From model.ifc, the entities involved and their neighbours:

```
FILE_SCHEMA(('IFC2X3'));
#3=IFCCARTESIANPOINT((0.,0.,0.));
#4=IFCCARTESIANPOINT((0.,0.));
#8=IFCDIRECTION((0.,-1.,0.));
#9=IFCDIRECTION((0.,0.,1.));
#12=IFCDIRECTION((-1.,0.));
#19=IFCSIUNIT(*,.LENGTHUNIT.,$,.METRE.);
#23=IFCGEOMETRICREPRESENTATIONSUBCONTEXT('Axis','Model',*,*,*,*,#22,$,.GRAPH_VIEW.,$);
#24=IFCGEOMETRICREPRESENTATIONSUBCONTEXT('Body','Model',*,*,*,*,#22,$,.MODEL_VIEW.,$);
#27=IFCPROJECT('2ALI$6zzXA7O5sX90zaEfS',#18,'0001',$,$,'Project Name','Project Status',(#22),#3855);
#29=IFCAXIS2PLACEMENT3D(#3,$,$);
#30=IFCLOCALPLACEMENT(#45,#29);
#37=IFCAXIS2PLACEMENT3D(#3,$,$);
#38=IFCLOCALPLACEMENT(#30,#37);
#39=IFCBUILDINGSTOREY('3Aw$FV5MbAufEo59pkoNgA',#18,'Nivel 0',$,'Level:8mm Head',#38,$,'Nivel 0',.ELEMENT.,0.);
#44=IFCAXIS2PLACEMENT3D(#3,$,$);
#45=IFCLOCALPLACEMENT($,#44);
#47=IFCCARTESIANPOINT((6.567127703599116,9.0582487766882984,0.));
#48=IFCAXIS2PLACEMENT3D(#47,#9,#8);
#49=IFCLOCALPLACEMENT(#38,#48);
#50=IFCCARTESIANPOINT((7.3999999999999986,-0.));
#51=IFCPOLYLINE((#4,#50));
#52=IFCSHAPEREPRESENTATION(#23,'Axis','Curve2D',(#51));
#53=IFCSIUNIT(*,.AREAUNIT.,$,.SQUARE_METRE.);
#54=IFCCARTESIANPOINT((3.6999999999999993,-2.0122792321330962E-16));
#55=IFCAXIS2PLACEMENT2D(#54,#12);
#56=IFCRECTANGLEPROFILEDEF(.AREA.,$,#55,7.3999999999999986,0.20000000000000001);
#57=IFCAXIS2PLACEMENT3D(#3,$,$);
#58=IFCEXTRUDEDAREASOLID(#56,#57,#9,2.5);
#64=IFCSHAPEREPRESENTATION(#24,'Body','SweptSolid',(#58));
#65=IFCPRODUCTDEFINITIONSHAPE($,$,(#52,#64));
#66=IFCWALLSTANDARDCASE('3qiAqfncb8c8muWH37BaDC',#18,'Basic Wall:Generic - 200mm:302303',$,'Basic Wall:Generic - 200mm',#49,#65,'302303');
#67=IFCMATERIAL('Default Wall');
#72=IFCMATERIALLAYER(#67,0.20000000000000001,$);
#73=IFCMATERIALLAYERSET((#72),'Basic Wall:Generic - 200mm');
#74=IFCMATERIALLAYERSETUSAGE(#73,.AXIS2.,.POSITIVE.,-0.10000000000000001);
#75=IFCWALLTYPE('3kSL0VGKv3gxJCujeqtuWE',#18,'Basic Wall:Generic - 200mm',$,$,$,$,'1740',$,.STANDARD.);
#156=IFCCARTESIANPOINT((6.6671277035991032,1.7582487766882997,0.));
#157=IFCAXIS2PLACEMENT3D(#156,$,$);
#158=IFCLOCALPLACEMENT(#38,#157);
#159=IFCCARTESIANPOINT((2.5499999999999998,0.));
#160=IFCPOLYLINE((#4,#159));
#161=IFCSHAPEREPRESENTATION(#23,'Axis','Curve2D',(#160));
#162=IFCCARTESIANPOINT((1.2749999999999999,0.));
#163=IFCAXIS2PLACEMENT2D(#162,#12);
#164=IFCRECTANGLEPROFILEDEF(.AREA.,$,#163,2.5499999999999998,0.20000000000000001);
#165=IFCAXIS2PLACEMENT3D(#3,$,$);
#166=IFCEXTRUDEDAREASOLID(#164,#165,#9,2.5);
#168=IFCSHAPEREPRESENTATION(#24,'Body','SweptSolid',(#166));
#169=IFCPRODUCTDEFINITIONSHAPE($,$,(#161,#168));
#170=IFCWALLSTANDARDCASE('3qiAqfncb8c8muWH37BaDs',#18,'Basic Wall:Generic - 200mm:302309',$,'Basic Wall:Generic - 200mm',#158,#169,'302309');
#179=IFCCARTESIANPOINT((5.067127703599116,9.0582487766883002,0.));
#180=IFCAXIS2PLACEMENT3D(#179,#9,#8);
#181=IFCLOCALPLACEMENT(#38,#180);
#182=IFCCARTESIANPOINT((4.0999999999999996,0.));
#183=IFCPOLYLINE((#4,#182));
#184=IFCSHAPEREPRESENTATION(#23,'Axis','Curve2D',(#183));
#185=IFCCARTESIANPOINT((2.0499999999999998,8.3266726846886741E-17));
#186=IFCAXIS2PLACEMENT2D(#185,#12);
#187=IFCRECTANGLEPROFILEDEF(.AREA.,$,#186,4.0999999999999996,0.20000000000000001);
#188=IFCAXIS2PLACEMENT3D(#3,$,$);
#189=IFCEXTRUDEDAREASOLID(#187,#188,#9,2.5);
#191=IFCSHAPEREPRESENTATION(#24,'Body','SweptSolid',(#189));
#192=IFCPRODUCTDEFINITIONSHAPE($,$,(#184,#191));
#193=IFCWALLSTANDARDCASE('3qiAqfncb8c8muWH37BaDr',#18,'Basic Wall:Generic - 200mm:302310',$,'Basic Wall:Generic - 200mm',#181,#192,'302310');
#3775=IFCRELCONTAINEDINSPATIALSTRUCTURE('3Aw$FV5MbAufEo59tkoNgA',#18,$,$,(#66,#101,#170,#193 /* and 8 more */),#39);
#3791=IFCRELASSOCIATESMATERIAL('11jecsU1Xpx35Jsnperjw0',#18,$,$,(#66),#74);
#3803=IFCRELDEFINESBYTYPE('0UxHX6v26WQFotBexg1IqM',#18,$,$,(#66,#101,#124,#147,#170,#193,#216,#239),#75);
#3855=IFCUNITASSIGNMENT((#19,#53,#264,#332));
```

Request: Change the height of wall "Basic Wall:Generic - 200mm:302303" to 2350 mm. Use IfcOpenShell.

```python
import ifcopenshell
import ifcopenshell.geom
import ifcopenshell.util.representation
import ifcopenshell.util.shape
import ifcopenshell.util.unit

model = ifcopenshell.open("model.ifc")
unit_scale = ifcopenshell.util.unit.calculate_unit_scale(model)
settings = ifcopenshell.geom.settings()


def volume(element):
    """Net volume in cubic metres, openings subtracted."""
    shape = ifcopenshell.geom.create_shape(settings, element)
    return ifcopenshell.util.shape.get_volume(shape.geometry)


wall = model.by_id(66)
before = volume(wall)

body = ifcopenshell.util.representation.get_representation(wall, "Model", "Body")
solid = body.Items[0]
old_height = solid.Depth
solid.Depth = 2.35 / unit_scale
after = volume(wall)

print(f"height {old_height:g} -> {solid.Depth:g}, volume {before:.3f} -> {after:.3f} m3")

model.write("model_v2.ifc")
```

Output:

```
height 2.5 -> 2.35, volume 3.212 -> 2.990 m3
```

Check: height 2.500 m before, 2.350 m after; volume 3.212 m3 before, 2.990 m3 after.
